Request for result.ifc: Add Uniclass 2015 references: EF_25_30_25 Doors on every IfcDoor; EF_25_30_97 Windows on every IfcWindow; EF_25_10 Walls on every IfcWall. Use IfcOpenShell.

First a look at what the model holds.

```python
import ifcopenshell

model = ifcopenshell.open("result.ifc")
print(model.schema)
print("classifications:", [c.Name for c in model.by_type("IfcClassification")])
for ifc_class in ("IfcDoor", "IfcRoof", "IfcStair", "IfcWall", "IfcWindow"):
    print(ifc_class, len(model.by_type(ifc_class)))
```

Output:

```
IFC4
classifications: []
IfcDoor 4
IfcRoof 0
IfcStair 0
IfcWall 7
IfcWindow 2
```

```python
import ifcopenshell
import ifcopenshell.api.classification

model = ifcopenshell.open("result.ifc")

system = ifcopenshell.api.classification.add_classification(model, classification="Uniclass 2015")

codes = {
    "IfcDoor": ("EF_25_30_25", "Doors"),
    "IfcWindow": ("EF_25_30_97", "Windows"),
    "IfcWall": ("EF_25_10", "Walls"),
}
for ifc_class, (code, name) in codes.items():
    products = model.by_type(ifc_class)
    ifcopenshell.api.classification.add_reference(
        model, products=products, classification=system, identification=code, name=name
    )
    print(code, len(products))

model.write("result_v2.ifc")
```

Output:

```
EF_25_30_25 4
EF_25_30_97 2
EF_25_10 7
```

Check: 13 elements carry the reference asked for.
